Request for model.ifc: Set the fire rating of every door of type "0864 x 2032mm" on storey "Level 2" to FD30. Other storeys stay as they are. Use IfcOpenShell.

First a look at what the model holds.

```python
import ifcopenshell
import ifcopenshell.util.element

model = ifcopenshell.open("model.ifc")
print(model.schema)
storey = next(s for s in model.by_type("IfcBuildingStorey") if s.Name == "Level 2")
doors = [e for e in ifcopenshell.util.element.get_decomposition(storey) if e.is_a("IfcDoor")]
seen = {}
for e in doors:
    element_type = ifcopenshell.util.element.get_type(e)
    key = (element_type.Name if element_type != e and element_type else None, ifcopenshell.util.element.get_pset(e, "Pset_DoorCommon", "FireRating"))
    seen[key] = seen.get(key, 0) + 1
for (name, value), count in sorted(seen.items(), key=str):
    print(count, "x", name, "|", value)
```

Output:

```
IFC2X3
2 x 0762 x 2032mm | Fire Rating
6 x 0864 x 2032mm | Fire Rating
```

```python
import ifcopenshell
import ifcopenshell.api.pset
import ifcopenshell.util.element

model = ifcopenshell.open("model.ifc")

storey = next(s for s in model.by_type("IfcBuildingStorey") if s.Name == "Level 2")
doors = [e for e in ifcopenshell.util.element.get_decomposition(storey) if e.is_a("IfcDoor")]

count = 0
for e in doors:
    element_type = ifcopenshell.util.element.get_type(e)
    if element_type in (None, e) or element_type.Name != "0864 x 2032mm":
        continue
    # add_pset returns the element's existing set when there is one.
    pset = ifcopenshell.api.pset.add_pset(model, product=e, name="Pset_DoorCommon")
    ifcopenshell.api.pset.edit_pset(model, pset=pset, properties={"FireRating": "FD30"})
    count += 1

print(count, "doors updated")

model.write("model_updated.ifc")
```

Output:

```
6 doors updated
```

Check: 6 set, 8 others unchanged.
